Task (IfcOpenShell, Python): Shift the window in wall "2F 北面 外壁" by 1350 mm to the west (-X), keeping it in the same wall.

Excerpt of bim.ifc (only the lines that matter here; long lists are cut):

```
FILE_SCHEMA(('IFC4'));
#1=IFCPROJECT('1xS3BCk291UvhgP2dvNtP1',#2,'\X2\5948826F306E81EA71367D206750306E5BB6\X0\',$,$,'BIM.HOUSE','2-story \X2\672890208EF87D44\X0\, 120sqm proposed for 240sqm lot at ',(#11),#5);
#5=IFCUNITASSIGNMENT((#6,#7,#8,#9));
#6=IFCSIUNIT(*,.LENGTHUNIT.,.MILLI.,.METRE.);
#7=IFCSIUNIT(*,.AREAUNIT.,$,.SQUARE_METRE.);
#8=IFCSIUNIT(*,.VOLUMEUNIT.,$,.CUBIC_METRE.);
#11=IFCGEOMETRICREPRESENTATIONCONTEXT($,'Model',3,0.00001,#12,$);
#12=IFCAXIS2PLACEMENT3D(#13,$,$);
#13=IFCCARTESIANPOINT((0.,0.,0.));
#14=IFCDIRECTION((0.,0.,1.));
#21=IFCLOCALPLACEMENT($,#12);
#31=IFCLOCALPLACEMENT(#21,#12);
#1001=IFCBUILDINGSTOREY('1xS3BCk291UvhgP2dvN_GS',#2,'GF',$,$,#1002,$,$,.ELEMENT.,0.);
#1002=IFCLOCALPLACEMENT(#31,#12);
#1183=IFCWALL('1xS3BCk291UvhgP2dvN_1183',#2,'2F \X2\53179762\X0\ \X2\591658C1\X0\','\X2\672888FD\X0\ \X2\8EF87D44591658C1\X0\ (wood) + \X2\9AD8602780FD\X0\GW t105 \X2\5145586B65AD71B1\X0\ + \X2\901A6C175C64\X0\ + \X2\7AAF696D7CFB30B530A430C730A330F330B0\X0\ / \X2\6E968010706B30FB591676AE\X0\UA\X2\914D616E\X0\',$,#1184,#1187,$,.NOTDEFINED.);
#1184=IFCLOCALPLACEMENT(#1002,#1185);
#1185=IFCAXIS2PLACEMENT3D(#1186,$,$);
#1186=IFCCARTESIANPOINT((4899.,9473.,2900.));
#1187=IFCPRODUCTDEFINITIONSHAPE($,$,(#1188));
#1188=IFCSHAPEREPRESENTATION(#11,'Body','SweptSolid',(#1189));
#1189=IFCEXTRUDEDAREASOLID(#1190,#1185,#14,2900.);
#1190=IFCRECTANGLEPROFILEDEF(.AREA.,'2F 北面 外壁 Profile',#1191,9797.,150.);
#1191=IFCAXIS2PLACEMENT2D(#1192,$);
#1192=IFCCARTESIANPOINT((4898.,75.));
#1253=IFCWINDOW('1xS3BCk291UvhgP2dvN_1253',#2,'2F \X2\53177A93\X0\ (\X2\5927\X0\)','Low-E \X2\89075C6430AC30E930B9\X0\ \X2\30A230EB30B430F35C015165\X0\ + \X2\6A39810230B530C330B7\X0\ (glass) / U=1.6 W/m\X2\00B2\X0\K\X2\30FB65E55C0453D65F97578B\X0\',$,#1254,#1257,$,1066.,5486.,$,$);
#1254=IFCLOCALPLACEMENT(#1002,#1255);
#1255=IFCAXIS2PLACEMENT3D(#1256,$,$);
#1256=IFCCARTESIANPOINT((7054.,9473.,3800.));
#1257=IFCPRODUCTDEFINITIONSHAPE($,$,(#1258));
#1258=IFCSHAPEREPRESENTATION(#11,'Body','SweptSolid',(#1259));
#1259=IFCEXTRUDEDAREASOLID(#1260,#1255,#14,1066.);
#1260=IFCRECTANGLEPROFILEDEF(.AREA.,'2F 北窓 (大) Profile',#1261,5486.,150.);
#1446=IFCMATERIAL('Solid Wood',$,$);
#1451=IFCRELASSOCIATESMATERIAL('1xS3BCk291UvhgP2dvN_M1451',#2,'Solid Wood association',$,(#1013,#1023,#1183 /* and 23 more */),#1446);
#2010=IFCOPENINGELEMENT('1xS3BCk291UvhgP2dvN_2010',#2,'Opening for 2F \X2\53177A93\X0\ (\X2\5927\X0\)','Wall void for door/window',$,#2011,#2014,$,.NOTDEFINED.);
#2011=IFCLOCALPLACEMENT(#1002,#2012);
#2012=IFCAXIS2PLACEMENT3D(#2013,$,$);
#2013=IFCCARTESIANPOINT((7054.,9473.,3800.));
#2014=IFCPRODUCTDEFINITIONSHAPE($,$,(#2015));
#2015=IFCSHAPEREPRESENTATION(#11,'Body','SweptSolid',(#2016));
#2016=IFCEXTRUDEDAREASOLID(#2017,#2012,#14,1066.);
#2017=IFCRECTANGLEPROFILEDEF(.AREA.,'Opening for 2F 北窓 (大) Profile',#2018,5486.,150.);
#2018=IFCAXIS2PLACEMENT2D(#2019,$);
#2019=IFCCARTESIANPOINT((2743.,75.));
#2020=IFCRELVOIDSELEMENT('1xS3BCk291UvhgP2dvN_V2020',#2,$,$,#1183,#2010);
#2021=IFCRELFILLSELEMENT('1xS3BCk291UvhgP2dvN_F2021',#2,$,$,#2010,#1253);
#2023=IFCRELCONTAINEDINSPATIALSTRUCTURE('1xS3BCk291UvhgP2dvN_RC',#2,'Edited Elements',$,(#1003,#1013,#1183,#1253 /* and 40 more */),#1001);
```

```python
import ifcopenshell
import ifcopenshell.api.geometry
import ifcopenshell.util.placement
import ifcopenshell.util.unit

model = ifcopenshell.open("bim.ifc")
unit_scale = ifcopenshell.util.unit.calculate_unit_scale(model)

window = model.by_guid("1xS3BCk291UvhgP2dvN_1253")
opening = window.FillsVoids[0].RelatingOpeningElement
wall = opening.VoidsElements[0].RelatingBuildingElement

wall_matrix = ifcopenshell.util.placement.get_local_placement(wall.ObjectPlacement)
shift = wall_matrix[:3, 0] * -1.35 / unit_scale
before = ifcopenshell.util.placement.get_local_placement(window.ObjectPlacement)[:3, 3].copy()

# The window is not placed relative to its opening, so move both.
for product in (opening, window):
    matrix = ifcopenshell.util.placement.get_local_placement(product.ObjectPlacement)
    matrix[:3, 3] += shift
    ifcopenshell.api.geometry.edit_object_placement(model, product=product, matrix=matrix, is_si=False)

after = ifcopenshell.util.placement.get_local_placement(window.ObjectPlacement)[:3, 3]
print("window moved by", (after - before).round(3) + 0.0)

model.write("bim_edited.ifc")
```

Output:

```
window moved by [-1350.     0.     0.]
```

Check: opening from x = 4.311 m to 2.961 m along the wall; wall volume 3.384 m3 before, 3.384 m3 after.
